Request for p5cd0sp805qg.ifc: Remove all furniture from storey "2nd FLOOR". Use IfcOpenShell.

First a look at what the model holds.

```python
import ifcopenshell
import ifcopenshell.util.element

model = ifcopenshell.open("p5cd0sp805qg.ifc")
print(model.schema)
storey = next(s for s in model.by_type("IfcBuildingStorey") if s.Name == "2nd FLOOR")
furniture = [e for e in ifcopenshell.util.element.get_decomposition(storey) if e.is_a("IfcFurnishingElement")]
seen = {}
for e in furniture:
    element_type = ifcopenshell.util.element.get_type(e)
    name = element_type.Name if element_type not in (None, e) else None
    seen[name] = seen.get(name, 0) + 1
for name, count in sorted(seen.items(), key=str):
    print(count, "x", name)
```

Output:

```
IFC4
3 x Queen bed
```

```python
import ifcopenshell
import ifcopenshell.api.root
import ifcopenshell.util.element

model = ifcopenshell.open("p5cd0sp805qg.ifc")

storey = next(s for s in model.by_type("IfcBuildingStorey") if s.Name == "2nd FLOOR")
furniture = [e for e in ifcopenshell.util.element.get_decomposition(storey) if e.is_a("IfcFurnishingElement")]

for e in furniture:
    ifcopenshell.api.root.remove_product(model, product=e)
print(len(furniture), "removed")

model.write("p5cd0sp805qg_rev.ifc")
```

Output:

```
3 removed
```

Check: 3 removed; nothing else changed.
